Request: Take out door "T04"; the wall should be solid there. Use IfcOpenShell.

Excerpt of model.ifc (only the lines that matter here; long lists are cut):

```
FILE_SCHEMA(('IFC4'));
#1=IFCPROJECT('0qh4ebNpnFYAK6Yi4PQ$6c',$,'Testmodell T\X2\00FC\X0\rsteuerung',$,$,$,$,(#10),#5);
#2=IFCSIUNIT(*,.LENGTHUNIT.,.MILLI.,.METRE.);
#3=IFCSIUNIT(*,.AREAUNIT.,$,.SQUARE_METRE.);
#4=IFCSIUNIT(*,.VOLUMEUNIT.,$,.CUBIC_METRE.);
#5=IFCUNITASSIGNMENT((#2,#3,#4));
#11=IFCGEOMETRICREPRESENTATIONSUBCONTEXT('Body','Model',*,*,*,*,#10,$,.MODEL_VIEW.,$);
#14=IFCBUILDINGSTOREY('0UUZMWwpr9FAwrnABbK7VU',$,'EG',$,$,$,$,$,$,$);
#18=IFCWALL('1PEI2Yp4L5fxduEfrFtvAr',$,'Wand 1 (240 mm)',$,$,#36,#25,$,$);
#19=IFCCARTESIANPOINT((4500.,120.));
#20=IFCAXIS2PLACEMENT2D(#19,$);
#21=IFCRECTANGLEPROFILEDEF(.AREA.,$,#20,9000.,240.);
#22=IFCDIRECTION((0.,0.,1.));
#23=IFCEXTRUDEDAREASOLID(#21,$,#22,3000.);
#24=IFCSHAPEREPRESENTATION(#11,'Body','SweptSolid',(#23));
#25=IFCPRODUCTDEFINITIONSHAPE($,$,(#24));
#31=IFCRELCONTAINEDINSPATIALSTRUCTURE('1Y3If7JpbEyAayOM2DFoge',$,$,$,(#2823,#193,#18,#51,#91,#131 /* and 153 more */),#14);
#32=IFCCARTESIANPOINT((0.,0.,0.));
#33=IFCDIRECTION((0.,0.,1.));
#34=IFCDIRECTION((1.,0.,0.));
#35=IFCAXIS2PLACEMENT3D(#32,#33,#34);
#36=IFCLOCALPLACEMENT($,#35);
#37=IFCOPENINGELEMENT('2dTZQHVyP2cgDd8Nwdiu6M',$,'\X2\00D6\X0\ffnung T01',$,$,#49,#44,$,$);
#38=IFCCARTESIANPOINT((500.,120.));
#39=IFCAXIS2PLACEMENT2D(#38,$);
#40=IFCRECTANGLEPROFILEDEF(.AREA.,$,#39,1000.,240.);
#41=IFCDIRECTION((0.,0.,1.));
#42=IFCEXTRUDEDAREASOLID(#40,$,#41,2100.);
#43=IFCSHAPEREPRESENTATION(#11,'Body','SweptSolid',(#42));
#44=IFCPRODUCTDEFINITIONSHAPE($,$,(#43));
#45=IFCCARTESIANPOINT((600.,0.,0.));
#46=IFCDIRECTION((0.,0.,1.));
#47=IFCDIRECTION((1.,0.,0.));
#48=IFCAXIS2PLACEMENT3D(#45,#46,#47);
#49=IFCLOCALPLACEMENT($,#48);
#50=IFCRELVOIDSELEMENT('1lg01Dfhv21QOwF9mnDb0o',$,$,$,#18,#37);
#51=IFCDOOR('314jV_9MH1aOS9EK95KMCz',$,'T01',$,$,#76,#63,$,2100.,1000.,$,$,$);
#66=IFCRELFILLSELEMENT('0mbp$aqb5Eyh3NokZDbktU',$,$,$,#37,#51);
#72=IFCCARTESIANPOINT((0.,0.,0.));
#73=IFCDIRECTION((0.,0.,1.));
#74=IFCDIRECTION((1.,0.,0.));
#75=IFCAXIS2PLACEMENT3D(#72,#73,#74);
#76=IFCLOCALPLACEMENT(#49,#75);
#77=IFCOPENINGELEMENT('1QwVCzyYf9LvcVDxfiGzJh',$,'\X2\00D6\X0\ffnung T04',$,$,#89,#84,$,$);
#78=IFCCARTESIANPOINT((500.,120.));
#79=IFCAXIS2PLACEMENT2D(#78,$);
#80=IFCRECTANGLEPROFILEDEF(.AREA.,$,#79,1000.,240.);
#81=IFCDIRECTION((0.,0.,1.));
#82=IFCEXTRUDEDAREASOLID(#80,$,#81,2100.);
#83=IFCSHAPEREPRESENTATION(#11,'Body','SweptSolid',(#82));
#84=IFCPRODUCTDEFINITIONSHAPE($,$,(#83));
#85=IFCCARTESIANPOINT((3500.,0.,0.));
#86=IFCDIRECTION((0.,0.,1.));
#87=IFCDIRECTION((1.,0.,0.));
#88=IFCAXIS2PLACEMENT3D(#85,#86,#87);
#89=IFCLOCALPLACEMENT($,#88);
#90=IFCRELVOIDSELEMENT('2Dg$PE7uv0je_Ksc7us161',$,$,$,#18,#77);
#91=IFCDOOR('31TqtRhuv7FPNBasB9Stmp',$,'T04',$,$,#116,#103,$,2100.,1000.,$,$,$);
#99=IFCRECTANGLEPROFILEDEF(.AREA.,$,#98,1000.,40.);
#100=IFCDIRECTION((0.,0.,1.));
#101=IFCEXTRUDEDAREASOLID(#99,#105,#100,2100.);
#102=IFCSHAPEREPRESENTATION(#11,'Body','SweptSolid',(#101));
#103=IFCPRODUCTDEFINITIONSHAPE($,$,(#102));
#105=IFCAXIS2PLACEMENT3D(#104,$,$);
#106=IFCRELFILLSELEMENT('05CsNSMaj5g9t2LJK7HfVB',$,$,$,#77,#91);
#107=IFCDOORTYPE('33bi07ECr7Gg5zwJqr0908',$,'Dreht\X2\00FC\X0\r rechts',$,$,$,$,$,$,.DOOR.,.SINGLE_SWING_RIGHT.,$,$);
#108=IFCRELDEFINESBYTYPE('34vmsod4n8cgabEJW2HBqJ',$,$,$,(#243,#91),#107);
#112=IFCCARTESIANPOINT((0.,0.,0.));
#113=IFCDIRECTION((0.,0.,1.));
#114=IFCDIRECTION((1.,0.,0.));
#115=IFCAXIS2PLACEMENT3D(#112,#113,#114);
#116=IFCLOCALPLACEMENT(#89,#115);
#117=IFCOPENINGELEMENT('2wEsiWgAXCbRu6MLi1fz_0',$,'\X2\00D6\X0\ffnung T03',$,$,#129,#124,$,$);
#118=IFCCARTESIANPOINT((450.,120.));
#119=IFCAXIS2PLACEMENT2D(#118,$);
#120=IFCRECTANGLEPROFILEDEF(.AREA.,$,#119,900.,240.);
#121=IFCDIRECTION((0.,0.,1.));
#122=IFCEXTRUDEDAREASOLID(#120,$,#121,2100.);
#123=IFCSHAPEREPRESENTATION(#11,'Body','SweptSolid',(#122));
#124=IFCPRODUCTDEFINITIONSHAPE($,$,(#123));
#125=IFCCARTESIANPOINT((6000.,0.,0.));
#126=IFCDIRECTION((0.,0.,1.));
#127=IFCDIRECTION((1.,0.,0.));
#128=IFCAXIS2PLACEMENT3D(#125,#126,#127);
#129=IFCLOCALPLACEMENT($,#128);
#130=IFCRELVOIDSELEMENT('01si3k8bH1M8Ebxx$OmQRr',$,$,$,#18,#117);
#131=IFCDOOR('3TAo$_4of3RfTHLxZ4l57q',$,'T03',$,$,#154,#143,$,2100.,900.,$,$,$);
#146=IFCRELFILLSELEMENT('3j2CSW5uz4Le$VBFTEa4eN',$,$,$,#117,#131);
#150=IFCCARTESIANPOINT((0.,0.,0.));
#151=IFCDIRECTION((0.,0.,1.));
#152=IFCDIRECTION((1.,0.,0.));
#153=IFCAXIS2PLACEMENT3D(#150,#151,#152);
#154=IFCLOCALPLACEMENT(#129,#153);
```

```python
import ifcopenshell
import ifcopenshell.api.feature
import ifcopenshell.api.root
import ifcopenshell.geom
import ifcopenshell.util.shape

model = ifcopenshell.open("model.ifc")
settings = ifcopenshell.geom.settings()


def volume(element):
    """Net volume in cubic metres, openings subtracted."""
    shape = ifcopenshell.geom.create_shape(settings, element)
    return ifcopenshell.util.shape.get_volume(shape.geometry)


door = model.by_guid("31TqtRhuv7FPNBasB9Stmp")
opening = door.FillsVoids[0].RelatingOpeningElement
wall = opening.VoidsElements[0].RelatingBuildingElement
before = volume(wall)

ifcopenshell.api.root.remove_product(model, product=door)
ifcopenshell.api.feature.remove_feature(model, feature=opening)

after = volume(wall)

print(f"wall volume {before:.3f} -> {after:.3f} m3")

model.write("model_v2.ifc")
```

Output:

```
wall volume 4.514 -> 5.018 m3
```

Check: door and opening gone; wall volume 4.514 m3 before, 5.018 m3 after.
